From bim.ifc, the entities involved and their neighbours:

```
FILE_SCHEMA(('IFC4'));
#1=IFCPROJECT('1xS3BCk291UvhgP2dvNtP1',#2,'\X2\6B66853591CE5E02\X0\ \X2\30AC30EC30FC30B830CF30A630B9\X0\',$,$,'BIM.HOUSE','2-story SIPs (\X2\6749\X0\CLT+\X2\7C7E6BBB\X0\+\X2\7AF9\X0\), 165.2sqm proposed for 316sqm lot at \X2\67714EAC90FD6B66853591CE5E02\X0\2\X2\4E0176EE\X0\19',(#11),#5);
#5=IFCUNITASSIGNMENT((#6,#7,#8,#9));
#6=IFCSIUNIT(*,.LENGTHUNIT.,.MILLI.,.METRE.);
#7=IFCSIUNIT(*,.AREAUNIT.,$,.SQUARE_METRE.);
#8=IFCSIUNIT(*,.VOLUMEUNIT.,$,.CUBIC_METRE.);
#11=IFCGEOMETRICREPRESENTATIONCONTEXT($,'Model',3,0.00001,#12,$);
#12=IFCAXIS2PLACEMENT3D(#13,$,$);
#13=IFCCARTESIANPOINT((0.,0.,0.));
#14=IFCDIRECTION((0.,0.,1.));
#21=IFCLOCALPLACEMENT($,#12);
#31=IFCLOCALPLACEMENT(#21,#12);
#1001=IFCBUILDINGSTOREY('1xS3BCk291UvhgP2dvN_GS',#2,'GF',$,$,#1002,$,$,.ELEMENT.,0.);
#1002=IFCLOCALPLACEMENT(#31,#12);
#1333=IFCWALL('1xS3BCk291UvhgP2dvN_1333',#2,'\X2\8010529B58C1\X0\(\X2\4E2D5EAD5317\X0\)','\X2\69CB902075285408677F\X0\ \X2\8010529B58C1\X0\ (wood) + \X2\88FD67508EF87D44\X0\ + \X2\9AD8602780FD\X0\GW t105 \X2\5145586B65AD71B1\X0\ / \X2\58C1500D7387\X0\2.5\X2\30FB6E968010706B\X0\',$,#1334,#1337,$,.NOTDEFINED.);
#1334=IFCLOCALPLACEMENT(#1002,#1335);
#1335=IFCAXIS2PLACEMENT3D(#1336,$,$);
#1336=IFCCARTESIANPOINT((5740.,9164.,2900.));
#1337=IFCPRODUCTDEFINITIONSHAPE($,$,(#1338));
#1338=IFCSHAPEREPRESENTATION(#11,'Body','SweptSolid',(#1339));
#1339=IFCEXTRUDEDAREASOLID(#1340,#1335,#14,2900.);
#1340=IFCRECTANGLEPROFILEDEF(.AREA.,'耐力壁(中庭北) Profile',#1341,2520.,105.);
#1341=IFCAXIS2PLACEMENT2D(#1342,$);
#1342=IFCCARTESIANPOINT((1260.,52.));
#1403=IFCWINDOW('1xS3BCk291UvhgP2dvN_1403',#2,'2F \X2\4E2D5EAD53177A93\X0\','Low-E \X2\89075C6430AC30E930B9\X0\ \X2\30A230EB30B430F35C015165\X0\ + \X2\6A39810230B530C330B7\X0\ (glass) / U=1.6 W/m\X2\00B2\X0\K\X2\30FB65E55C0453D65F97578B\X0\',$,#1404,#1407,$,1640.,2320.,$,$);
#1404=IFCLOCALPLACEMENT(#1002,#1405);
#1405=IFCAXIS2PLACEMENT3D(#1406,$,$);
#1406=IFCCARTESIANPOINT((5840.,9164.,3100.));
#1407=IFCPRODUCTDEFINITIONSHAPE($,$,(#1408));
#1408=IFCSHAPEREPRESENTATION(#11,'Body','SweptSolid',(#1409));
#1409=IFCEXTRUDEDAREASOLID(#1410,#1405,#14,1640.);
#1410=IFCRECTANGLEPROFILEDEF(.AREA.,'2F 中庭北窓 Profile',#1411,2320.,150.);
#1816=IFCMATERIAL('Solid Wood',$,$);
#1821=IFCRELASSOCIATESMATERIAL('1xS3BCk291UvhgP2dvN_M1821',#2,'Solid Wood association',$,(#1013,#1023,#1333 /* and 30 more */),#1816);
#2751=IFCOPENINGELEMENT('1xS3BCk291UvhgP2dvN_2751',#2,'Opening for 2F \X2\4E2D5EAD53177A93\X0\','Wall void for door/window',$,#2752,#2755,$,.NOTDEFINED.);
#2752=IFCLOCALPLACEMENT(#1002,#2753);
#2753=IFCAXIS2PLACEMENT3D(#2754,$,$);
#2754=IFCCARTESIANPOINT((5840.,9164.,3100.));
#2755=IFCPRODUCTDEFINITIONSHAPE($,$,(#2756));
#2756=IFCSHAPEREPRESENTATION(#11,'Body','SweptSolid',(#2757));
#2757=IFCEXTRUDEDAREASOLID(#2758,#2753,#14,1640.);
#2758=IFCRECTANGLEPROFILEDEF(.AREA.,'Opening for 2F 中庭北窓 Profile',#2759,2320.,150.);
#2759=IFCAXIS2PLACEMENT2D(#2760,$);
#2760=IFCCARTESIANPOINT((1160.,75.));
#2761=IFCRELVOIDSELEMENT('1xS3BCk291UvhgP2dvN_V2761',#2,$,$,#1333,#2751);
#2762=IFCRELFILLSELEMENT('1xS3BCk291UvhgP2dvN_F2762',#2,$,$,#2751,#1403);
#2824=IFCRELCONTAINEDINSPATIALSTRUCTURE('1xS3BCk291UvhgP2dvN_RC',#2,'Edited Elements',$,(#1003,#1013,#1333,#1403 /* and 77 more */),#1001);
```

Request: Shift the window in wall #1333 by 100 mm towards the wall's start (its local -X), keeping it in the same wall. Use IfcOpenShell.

```python
import ifcopenshell
import ifcopenshell.api.geometry
import ifcopenshell.util.placement

model = ifcopenshell.open("bim.ifc")

window = model.by_id(1403)
opening = window.FillsVoids[0].RelatingOpeningElement
wall = opening.VoidsElements[0].RelatingBuildingElement

wall_matrix = ifcopenshell.util.placement.get_local_placement(wall.ObjectPlacement)
shift = wall_matrix[:3, 0] * -100.0
before = ifcopenshell.util.placement.get_local_placement(window.ObjectPlacement)[:3, 3].copy()

# The window is not placed relative to its opening, so move both.
for product in (opening, window):
    matrix = ifcopenshell.util.placement.get_local_placement(product.ObjectPlacement)
    matrix[:3, 3] += shift
    ifcopenshell.api.geometry.edit_object_placement(model, product=product, matrix=matrix, is_si=False)

after = ifcopenshell.util.placement.get_local_placement(window.ObjectPlacement)[:3, 3]
print("window moved by", (after - before).round(3) + 0.0)

model.write("bim_updated.ifc")
```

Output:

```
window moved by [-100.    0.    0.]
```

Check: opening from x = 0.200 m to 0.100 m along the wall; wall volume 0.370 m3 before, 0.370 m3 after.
